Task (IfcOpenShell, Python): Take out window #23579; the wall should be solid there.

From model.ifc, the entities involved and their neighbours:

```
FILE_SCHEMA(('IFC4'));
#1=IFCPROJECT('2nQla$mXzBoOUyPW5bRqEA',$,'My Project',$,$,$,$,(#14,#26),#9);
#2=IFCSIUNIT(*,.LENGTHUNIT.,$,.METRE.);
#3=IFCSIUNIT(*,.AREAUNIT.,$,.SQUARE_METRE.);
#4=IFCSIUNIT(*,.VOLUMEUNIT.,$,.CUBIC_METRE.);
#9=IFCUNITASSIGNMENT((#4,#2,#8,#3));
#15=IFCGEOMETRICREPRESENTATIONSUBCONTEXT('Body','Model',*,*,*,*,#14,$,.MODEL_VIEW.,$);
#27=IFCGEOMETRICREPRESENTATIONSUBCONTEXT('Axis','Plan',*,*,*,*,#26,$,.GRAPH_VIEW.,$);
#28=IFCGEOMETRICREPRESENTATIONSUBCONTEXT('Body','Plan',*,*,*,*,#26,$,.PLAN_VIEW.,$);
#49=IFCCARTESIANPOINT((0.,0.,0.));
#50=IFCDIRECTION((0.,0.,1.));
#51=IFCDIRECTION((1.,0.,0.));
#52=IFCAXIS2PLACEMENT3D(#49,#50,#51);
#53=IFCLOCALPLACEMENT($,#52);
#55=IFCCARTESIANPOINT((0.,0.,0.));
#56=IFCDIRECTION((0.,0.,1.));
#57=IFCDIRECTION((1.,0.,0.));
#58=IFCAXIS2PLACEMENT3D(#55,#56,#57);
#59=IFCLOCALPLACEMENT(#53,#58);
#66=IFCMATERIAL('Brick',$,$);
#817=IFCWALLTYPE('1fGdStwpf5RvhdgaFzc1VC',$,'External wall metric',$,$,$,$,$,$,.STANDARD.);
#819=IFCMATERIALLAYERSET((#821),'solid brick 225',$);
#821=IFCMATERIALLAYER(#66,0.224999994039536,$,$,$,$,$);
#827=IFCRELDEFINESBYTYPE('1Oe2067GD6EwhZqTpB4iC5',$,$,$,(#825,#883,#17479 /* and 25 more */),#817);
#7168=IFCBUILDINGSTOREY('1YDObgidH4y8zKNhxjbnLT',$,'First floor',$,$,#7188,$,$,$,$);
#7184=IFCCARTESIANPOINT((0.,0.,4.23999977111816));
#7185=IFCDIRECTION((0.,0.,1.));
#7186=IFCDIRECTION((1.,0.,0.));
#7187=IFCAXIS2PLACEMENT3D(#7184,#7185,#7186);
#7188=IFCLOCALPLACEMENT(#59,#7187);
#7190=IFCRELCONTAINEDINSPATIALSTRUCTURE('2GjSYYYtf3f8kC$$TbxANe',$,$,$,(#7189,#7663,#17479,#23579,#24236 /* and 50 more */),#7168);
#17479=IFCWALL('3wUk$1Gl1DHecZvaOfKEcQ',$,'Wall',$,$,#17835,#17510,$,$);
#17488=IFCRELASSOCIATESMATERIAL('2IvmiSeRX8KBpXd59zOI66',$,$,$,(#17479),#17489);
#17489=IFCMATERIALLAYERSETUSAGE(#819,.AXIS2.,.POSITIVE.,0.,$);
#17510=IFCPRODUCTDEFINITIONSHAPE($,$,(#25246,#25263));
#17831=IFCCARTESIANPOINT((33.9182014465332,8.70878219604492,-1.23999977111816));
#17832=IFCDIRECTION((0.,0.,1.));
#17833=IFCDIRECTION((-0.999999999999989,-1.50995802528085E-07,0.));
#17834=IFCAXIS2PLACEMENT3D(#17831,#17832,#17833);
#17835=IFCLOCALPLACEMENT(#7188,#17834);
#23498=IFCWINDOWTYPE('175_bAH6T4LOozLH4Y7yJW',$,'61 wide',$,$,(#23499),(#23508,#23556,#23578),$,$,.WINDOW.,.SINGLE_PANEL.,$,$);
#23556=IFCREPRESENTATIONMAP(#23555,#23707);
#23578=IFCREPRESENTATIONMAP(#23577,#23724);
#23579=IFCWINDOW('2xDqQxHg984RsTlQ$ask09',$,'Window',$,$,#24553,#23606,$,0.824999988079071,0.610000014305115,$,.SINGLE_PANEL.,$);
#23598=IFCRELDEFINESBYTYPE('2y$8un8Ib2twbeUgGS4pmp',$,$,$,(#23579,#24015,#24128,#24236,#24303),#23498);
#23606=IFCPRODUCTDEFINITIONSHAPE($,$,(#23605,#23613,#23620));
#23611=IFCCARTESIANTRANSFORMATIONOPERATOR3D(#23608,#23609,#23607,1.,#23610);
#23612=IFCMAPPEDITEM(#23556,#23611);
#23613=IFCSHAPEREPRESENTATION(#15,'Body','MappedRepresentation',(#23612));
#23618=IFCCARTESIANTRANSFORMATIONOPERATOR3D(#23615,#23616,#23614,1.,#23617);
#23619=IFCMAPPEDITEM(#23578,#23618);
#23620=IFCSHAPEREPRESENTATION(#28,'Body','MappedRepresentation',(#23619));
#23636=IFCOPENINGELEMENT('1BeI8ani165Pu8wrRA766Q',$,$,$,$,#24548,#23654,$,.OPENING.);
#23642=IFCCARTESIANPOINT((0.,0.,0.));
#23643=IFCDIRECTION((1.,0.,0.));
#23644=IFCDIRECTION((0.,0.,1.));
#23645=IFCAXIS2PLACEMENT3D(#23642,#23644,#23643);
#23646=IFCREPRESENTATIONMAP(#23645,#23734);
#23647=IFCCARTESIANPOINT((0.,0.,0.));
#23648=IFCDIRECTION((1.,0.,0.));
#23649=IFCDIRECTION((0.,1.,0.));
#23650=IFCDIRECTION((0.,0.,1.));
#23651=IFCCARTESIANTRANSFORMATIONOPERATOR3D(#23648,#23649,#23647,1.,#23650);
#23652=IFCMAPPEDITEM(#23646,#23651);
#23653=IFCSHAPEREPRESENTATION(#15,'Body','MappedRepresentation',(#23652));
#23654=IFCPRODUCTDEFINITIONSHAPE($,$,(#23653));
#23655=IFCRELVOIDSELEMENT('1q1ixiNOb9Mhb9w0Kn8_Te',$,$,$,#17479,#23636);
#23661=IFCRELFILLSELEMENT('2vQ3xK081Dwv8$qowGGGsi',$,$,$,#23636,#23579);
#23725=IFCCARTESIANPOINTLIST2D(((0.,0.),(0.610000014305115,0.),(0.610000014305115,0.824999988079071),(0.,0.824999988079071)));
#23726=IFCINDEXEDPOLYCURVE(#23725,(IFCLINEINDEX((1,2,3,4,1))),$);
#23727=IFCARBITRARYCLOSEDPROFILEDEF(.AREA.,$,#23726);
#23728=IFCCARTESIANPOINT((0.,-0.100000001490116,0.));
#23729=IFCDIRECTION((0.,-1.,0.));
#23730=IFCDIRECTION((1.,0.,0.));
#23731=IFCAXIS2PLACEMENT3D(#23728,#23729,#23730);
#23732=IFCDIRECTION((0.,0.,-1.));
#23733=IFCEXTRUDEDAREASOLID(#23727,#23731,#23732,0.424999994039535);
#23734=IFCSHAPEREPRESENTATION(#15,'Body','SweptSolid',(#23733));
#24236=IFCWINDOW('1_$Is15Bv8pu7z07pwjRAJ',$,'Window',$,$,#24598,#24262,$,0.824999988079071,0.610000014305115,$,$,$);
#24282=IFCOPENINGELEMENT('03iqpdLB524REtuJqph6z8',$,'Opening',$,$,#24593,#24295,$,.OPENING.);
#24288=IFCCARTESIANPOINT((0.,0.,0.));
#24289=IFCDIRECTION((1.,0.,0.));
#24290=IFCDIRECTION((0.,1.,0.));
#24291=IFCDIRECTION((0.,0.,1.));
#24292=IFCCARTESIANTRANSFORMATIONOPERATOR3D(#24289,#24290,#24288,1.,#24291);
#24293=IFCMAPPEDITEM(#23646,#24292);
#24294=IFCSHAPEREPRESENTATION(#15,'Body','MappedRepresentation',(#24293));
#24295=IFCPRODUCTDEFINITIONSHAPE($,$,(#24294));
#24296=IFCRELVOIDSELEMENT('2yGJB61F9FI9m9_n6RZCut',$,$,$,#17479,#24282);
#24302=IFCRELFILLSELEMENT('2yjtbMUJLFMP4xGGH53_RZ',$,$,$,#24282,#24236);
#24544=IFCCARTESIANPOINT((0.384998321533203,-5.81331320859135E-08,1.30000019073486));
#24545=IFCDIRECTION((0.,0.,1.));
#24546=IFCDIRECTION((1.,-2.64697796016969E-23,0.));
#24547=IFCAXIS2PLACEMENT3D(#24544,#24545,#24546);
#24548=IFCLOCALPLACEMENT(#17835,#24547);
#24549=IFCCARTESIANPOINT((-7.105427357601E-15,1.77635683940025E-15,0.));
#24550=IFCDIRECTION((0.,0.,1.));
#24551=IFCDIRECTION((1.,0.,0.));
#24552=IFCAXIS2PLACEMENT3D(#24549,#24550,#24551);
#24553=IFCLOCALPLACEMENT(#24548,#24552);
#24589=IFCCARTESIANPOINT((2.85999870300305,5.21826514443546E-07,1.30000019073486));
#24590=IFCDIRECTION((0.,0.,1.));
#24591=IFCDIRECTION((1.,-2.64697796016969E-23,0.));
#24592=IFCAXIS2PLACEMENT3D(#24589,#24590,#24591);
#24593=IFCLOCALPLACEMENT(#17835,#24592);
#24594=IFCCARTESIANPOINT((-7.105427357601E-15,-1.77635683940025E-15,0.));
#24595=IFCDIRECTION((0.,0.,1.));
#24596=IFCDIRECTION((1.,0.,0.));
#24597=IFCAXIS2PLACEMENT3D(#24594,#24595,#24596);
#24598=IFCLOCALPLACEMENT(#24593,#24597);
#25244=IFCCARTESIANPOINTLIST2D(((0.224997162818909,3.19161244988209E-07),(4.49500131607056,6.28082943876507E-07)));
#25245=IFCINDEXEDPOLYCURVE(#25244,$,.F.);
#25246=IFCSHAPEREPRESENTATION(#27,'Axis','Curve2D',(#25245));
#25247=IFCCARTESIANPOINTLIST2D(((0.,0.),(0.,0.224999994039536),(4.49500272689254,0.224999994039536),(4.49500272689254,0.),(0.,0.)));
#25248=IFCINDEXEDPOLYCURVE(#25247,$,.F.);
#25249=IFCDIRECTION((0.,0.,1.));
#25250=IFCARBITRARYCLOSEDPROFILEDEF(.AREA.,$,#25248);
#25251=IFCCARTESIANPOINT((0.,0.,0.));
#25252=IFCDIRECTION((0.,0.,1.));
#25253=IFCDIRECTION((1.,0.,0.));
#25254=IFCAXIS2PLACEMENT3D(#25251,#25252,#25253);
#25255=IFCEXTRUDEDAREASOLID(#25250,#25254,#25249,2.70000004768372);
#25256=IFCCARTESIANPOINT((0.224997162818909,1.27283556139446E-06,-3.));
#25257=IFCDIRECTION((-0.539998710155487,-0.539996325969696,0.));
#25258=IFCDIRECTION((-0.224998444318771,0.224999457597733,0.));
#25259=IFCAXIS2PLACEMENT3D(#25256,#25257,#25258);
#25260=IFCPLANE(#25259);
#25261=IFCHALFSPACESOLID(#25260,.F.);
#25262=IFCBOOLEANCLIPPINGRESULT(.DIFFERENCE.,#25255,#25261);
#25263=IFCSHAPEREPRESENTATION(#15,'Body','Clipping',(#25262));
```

```python
import ifcopenshell
import ifcopenshell.api.feature
import ifcopenshell.api.root
import ifcopenshell.geom
import ifcopenshell.util.shape

model = ifcopenshell.open("model.ifc")
settings = ifcopenshell.geom.settings()


def volume(element):
    """Net volume in cubic metres, openings subtracted."""
    shape = ifcopenshell.geom.create_shape(settings, element)
    return ifcopenshell.util.shape.get_volume(shape.geometry)


window = model.by_guid("2xDqQxHg984RsTlQ$ask09")
opening = window.FillsVoids[0].RelatingOpeningElement
wall = opening.VoidsElements[0].RelatingBuildingElement
before = volume(wall)

ifcopenshell.api.root.remove_product(model, product=window)
ifcopenshell.api.feature.remove_feature(model, feature=opening)

after = volume(wall)

print(f"wall volume {before:.3f} -> {after:.3f} m3")

model.write("model_rev.ifc")
```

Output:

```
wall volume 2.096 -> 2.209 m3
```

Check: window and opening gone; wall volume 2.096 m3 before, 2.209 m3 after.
